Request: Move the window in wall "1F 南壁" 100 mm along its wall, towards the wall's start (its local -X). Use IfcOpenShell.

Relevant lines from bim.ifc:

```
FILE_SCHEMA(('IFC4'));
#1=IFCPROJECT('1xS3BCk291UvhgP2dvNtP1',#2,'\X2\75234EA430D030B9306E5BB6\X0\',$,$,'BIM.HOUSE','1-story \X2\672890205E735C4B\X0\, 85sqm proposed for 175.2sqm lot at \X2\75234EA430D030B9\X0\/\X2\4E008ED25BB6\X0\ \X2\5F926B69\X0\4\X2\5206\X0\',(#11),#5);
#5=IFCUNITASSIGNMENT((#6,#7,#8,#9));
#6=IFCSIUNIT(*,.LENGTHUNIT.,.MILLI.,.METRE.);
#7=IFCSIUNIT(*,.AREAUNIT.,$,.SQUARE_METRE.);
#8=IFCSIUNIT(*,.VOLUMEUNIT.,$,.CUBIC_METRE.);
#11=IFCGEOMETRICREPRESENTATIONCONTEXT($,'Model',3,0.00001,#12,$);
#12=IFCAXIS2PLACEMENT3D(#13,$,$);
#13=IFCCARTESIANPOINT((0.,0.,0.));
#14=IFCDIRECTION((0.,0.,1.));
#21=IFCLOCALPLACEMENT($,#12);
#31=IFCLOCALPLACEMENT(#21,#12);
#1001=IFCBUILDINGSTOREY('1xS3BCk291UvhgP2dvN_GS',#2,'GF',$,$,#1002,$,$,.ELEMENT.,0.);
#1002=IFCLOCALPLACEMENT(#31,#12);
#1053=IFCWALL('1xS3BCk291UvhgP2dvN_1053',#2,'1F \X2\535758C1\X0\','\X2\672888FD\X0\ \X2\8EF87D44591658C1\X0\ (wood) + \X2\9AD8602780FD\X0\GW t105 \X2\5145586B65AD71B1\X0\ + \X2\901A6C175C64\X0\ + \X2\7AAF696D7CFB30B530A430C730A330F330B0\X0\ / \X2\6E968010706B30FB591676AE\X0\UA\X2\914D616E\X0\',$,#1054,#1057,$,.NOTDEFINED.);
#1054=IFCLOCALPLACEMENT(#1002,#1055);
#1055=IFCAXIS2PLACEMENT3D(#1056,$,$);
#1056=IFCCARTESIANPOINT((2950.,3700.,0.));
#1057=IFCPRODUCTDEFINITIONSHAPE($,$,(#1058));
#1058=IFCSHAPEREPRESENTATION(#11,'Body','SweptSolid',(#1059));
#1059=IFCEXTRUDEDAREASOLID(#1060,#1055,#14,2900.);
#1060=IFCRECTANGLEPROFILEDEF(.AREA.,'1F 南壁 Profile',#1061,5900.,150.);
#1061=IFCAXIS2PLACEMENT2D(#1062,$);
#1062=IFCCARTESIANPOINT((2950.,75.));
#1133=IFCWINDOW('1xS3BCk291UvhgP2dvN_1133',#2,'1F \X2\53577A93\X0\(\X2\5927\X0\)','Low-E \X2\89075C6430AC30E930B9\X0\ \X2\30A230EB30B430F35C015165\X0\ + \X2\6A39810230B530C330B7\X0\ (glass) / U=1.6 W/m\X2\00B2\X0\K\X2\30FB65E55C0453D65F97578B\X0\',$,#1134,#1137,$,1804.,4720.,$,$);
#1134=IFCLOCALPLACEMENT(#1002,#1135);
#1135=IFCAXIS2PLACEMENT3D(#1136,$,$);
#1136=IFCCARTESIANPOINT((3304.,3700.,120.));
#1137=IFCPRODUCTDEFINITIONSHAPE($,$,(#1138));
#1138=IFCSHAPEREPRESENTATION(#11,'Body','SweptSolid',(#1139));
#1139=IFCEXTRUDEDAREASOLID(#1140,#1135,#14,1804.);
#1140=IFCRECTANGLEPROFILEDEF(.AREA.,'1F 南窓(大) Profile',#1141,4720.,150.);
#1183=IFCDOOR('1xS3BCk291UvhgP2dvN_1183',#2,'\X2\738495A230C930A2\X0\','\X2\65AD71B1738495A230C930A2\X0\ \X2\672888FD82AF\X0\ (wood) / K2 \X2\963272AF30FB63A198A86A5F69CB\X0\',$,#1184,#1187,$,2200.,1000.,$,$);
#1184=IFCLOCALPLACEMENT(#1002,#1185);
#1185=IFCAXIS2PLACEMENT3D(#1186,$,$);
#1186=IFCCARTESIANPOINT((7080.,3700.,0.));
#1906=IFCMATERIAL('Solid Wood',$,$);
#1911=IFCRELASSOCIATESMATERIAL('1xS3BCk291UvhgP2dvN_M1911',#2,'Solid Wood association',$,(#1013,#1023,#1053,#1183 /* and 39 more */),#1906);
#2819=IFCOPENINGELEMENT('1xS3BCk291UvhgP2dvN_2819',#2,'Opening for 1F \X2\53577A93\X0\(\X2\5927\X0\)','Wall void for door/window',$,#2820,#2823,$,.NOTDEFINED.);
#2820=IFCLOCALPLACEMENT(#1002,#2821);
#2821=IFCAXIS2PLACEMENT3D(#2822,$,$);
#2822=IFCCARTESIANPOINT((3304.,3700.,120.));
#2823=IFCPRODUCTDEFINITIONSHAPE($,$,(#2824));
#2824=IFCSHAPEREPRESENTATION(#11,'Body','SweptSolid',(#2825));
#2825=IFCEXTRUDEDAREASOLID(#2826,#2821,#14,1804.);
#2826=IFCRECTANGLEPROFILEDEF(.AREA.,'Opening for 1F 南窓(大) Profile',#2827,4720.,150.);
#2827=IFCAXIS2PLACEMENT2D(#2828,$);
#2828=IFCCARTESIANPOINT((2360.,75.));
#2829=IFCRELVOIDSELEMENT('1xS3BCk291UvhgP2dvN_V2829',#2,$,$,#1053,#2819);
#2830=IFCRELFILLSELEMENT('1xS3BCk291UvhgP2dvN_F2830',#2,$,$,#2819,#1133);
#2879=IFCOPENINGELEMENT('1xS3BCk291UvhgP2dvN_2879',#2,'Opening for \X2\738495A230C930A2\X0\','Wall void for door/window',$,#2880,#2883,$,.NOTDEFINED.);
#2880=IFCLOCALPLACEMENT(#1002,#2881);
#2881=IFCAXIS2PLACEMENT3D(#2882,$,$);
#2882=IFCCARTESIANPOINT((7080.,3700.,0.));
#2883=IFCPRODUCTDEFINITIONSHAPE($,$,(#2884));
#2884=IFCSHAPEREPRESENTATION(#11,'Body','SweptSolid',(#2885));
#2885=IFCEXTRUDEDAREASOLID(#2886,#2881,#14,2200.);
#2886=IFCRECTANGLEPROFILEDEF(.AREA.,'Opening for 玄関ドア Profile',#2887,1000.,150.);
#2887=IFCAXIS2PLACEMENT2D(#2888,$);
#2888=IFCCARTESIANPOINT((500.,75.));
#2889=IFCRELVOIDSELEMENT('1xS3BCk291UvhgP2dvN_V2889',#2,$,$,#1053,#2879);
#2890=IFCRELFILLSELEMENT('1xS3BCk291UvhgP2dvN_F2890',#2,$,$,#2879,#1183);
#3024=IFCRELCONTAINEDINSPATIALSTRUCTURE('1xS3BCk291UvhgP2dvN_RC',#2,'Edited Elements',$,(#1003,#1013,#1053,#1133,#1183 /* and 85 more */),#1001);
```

```python
import ifcopenshell
import ifcopenshell.api.geometry
import ifcopenshell.util.placement
import ifcopenshell.util.unit

model = ifcopenshell.open("bim.ifc")
unit_scale = ifcopenshell.util.unit.calculate_unit_scale(model)

window = model.by_id(1133)
opening = window.FillsVoids[0].RelatingOpeningElement
wall = opening.VoidsElements[0].RelatingBuildingElement

wall_matrix = ifcopenshell.util.placement.get_local_placement(wall.ObjectPlacement)
shift = wall_matrix[:3, 0] * -0.1 / unit_scale
before = ifcopenshell.util.placement.get_local_placement(window.ObjectPlacement)[:3, 3].copy()

# The window is not placed relative to its opening, so move both.
for product in (opening, window):
    matrix = ifcopenshell.util.placement.get_local_placement(product.ObjectPlacement)
    matrix[:3, 3] += shift
    ifcopenshell.api.geometry.edit_object_placement(model, product=product, matrix=matrix, is_si=False)

after = ifcopenshell.util.placement.get_local_placement(window.ObjectPlacement)[:3, 3]
print("window moved by", (after - before).round(3) + 0.0)

model.write("bim-out.ifc")
```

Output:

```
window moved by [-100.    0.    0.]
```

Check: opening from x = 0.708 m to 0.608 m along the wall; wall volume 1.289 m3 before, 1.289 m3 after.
